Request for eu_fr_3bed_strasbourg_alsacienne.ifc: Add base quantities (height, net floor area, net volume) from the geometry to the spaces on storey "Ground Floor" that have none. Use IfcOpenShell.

First a look at what the model holds.

```python
import ifcopenshell
import ifcopenshell.util.element
import ifcopenshell.util.unit

model = ifcopenshell.open("eu_fr_3bed_strasbourg_alsacienne.ifc")
print(model.schema)
for unit_type in ("LENGTHUNIT", "AREAUNIT", "VOLUMEUNIT"):
    print(unit_type, ifcopenshell.util.unit.calculate_unit_scale(model, unit_type))
storey = next(s for s in model.by_type("IfcBuildingStorey") if s.Name == "Ground Floor")
spaces = [e for e in ifcopenshell.util.element.get_decomposition(storey) if e.is_a("IfcSpace")]
for e in sorted(spaces, key=lambda e: e.id()):
    print(e.id(), e.is_a(), e.Name, list(ifcopenshell.util.element.get_psets(e, qtos_only=True)), sep=" | ")
```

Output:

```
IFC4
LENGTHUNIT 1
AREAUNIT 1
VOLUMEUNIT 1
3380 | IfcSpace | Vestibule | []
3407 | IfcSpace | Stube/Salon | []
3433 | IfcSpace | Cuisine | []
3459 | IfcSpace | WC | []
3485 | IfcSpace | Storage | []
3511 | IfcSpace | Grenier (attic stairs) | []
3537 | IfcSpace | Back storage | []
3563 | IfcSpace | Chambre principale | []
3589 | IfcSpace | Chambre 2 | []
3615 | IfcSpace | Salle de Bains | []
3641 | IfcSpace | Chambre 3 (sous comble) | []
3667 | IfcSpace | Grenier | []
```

```python
import ifcopenshell
import ifcopenshell.api.pset
import ifcopenshell.geom
import ifcopenshell.util.element
import ifcopenshell.util.shape
import ifcopenshell.util.unit

model = ifcopenshell.open("eu_fr_3bed_strasbourg_alsacienne.ifc")
unit_scale = ifcopenshell.util.unit.calculate_unit_scale(model)
area_scale = ifcopenshell.util.unit.calculate_unit_scale(model, "AREAUNIT")
volume_scale = ifcopenshell.util.unit.calculate_unit_scale(model, "VOLUMEUNIT")
settings = ifcopenshell.geom.settings()

storey = next(s for s in model.by_type("IfcBuildingStorey") if s.Name == "Ground Floor")
spaces = [e for e in ifcopenshell.util.element.get_decomposition(storey) if e.is_a("IfcSpace")]

for e in sorted(spaces, key=lambda e: e.id()):
    if ifcopenshell.util.element.get_psets(e, qtos_only=True, should_inherit=False):
        continue
    # Geometry comes back in metres, in the element's own axes.
    shape = ifcopenshell.geom.create_shape(settings, e)
    values = {
        "Height": ifcopenshell.util.shape.get_z(shape.geometry) / unit_scale,
        "NetFloorArea": ifcopenshell.util.shape.get_footprint_area(shape.geometry) / area_scale,
        "NetVolume": ifcopenshell.util.shape.get_volume(shape.geometry) / volume_scale,
    }
    qto = ifcopenshell.api.pset.add_qto(model, product=e, name="Qto_SpaceBaseQuantities")
    ifcopenshell.api.pset.edit_qto(model, qto=qto, properties=values)
    print(e.id(), {k: round(v, 3) for k, v in values.items()})

model.write("eu_fr_3bed_strasbourg_alsacienne_rev.ifc")
```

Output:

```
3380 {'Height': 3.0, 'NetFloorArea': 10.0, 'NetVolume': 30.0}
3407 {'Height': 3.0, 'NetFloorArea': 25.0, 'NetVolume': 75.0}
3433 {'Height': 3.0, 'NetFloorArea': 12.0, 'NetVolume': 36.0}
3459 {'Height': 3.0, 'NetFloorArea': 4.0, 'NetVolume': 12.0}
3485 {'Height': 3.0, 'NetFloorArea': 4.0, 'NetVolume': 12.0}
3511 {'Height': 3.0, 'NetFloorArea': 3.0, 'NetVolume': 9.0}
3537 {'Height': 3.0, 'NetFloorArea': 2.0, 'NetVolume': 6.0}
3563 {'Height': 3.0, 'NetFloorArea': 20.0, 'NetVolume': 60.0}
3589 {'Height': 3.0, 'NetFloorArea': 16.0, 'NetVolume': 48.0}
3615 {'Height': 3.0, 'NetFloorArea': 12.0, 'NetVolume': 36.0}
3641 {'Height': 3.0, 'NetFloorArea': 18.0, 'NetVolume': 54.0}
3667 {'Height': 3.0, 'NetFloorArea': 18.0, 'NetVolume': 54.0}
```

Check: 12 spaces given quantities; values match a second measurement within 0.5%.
